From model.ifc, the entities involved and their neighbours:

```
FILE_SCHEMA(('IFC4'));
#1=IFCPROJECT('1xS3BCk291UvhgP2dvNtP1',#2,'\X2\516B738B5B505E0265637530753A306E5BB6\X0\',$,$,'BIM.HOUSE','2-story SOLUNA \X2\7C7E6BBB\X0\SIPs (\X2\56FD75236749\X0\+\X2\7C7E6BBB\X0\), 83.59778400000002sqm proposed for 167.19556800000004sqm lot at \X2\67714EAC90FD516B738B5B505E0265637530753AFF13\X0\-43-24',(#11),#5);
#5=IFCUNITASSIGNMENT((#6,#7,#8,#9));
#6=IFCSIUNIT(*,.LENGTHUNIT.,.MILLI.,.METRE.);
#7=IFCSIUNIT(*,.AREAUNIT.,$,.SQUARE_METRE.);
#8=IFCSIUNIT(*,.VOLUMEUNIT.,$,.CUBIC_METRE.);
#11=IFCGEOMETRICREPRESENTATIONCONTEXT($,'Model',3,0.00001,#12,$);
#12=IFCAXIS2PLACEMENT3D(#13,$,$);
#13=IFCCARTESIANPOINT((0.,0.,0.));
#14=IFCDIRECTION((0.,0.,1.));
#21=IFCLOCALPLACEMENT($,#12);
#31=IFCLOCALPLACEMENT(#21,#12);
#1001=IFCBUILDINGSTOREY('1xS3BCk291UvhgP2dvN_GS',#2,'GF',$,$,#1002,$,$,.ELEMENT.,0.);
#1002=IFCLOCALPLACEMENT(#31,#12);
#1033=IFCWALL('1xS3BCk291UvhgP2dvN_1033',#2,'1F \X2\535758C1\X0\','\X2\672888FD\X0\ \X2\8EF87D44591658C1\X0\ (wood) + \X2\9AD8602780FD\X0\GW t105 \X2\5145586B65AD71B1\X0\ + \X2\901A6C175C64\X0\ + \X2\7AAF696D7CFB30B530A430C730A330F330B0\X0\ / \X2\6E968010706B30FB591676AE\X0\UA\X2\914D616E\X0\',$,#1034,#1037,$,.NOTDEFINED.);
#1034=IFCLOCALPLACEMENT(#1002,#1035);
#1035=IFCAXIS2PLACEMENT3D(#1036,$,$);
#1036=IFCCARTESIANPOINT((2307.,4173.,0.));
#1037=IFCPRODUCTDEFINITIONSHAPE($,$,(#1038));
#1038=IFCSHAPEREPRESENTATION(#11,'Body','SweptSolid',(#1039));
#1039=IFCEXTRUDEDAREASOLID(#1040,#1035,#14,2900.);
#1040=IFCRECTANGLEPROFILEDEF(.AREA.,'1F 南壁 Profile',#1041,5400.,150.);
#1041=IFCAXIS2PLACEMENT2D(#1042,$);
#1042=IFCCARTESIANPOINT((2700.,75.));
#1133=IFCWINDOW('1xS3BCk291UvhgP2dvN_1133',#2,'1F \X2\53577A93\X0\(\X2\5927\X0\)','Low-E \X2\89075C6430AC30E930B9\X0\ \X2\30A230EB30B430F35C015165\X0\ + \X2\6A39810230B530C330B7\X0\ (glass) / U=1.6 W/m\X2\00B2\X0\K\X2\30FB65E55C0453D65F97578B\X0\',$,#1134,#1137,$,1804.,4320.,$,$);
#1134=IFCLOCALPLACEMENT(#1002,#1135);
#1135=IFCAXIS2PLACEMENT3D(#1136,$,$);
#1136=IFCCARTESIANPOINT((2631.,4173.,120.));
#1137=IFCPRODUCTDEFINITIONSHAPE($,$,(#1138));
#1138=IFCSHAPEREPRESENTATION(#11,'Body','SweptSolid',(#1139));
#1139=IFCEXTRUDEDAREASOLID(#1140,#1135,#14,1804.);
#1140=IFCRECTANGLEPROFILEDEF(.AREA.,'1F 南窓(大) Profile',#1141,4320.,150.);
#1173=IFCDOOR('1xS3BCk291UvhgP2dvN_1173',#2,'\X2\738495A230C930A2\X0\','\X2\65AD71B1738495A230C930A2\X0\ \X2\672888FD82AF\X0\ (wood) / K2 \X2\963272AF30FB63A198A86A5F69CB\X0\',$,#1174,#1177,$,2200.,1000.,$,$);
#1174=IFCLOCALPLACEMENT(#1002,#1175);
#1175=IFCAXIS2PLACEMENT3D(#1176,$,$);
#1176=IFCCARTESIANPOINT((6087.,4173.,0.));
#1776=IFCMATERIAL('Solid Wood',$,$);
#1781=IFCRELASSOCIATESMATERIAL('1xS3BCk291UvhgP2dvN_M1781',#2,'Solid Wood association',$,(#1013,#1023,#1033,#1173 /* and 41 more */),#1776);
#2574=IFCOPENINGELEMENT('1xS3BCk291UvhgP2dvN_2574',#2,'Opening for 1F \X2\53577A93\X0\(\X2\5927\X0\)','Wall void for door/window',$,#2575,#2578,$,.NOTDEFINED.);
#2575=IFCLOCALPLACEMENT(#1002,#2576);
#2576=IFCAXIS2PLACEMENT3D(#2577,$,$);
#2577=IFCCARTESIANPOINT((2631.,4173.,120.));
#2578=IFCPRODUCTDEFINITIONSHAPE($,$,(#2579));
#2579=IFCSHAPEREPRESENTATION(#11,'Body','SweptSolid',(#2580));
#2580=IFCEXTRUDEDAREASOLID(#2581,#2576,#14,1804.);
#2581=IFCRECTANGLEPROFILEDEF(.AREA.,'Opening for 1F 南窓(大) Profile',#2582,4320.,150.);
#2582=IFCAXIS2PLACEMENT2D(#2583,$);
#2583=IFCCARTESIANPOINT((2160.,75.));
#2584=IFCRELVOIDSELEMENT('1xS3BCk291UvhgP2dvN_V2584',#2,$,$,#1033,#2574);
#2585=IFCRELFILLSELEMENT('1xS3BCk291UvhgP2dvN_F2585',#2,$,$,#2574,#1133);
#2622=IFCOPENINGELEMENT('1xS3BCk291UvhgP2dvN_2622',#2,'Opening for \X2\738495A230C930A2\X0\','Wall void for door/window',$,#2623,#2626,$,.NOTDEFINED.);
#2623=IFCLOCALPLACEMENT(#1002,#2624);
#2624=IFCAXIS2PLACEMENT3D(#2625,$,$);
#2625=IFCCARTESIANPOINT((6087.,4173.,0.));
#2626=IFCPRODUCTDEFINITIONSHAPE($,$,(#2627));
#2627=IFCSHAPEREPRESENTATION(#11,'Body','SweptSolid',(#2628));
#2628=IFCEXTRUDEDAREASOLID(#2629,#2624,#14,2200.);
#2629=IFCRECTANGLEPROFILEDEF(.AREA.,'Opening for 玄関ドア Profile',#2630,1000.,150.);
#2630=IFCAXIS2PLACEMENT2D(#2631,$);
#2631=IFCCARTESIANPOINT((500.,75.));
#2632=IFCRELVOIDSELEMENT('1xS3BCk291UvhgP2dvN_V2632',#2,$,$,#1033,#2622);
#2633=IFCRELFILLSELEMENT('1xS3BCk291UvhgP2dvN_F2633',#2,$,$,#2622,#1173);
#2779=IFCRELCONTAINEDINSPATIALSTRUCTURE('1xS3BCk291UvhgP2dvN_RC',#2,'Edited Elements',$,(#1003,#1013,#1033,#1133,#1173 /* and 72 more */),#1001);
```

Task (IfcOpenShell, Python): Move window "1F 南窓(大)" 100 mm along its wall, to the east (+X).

```python
import ifcopenshell
import ifcopenshell.api.geometry
import ifcopenshell.util.placement
import ifcopenshell.util.unit

model = ifcopenshell.open("model.ifc")
unit_scale = ifcopenshell.util.unit.calculate_unit_scale(model)

window = model.by_guid("1xS3BCk291UvhgP2dvN_1133")
opening = window.FillsVoids[0].RelatingOpeningElement
wall = opening.VoidsElements[0].RelatingBuildingElement

wall_matrix = ifcopenshell.util.placement.get_local_placement(wall.ObjectPlacement)
shift = wall_matrix[:3, 0] * 0.1 / unit_scale
before = ifcopenshell.util.placement.get_local_placement(window.ObjectPlacement)[:3, 3].copy()

# The window is not placed relative to its opening, so move both.
for product in (opening, window):
    matrix = ifcopenshell.util.placement.get_local_placement(product.ObjectPlacement)
    matrix[:3, 3] += shift
    ifcopenshell.api.geometry.edit_object_placement(model, product=product, matrix=matrix, is_si=False)

after = ifcopenshell.util.placement.get_local_placement(window.ObjectPlacement)[:3, 3]
print("window moved by", (after - before).round(3) + 0.0)

model.write("model_v2.ifc")
```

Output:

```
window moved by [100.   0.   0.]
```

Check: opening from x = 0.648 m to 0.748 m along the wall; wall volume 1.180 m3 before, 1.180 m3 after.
